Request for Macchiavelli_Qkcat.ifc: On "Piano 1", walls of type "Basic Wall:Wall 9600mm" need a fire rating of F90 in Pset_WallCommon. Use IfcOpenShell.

First a look at what the model holds.

```python
import ifcopenshell
import ifcopenshell.util.element

model = ifcopenshell.open("Macchiavelli_Qkcat.ifc")
print(model.schema)
storey = next(s for s in model.by_type("IfcBuildingStorey") if s.Name == "Piano 1")
walls = [e for e in ifcopenshell.util.element.get_decomposition(storey) if e.is_a("IfcWall")]
seen = {}
for e in walls:
    element_type = ifcopenshell.util.element.get_type(e)
    key = (element_type.Name if element_type != e and element_type else None, ifcopenshell.util.element.get_pset(e, "Pset_WallCommon", "FireRating"))
    seen[key] = seen.get(key, 0) + 1
for (name, value), count in sorted(seen.items(), key=str):
    print(count, "x", name, "|", value)
```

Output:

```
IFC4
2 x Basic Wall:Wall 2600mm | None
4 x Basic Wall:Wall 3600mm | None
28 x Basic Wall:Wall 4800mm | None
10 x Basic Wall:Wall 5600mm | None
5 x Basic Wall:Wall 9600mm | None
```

```python
import ifcopenshell
import ifcopenshell.api.pset
import ifcopenshell.util.element

model = ifcopenshell.open("Macchiavelli_Qkcat.ifc")

storey = next(s for s in model.by_type("IfcBuildingStorey") if s.Name == "Piano 1")
walls = [e for e in ifcopenshell.util.element.get_decomposition(storey) if e.is_a("IfcWall")]

count = 0
for e in walls:
    element_type = ifcopenshell.util.element.get_type(e)
    if element_type in (None, e) or element_type.Name != "Basic Wall:Wall 9600mm":
        continue
    # add_pset returns the element's existing set when there is one.
    pset = ifcopenshell.api.pset.add_pset(model, product=e, name="Pset_WallCommon")
    ifcopenshell.api.pset.edit_pset(model, pset=pset, properties={"FireRating": "F90"})
    count += 1

print(count, "walls updated")

model.write("Macchiavelli_Qkcat_edited.ifc")
```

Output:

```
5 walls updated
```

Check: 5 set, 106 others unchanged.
